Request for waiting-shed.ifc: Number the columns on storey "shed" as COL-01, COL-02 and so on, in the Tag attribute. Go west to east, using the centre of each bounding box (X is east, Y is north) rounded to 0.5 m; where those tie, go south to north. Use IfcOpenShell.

First a look at what the model holds.

```python
import ifcopenshell
import ifcopenshell.util.element
import ifcopenshell.util.placement

model = ifcopenshell.open("waiting-shed.ifc")
print(model.schema)
storey = next(s for s in model.by_type("IfcBuildingStorey") if s.Name == "shed")
columns = [e for e in ifcopenshell.util.element.get_decomposition(storey) if e.is_a("IfcColumn")]
for e in sorted(columns, key=lambda e: e.id()):
    origin = ifcopenshell.util.placement.get_local_placement(e.ObjectPlacement)[:3, 3]
    print(e.id(), e.Tag, e.Name, origin.round(2) + 0.0, sep=" | ")
```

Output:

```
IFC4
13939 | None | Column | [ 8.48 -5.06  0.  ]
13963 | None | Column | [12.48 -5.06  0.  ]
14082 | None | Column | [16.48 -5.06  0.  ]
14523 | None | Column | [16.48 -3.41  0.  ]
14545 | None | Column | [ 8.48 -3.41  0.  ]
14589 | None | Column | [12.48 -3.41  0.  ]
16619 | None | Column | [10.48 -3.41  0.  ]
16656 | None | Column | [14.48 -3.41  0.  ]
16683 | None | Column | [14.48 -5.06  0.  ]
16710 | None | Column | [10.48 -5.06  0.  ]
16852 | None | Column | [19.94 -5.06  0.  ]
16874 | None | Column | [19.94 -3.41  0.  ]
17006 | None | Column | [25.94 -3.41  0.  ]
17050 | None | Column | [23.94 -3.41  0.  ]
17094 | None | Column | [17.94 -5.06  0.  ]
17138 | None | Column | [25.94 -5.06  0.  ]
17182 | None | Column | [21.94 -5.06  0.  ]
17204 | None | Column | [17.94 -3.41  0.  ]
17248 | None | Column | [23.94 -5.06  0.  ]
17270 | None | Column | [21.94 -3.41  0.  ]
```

```python
import ifcopenshell
import ifcopenshell.geom
import ifcopenshell.util.element
import ifcopenshell.util.shape

model = ifcopenshell.open("waiting-shed.ifc")
settings = ifcopenshell.geom.settings()
settings.set("use-world-coords", True)


def centre(element):
    shape = ifcopenshell.geom.create_shape(settings, element)
    return ifcopenshell.util.shape.get_bbox_centroid(shape.geometry)


storey = next(s for s in model.by_type("IfcBuildingStorey") if s.Name == "shed")
columns = [e for e in ifcopenshell.util.element.get_decomposition(storey) if e.is_a("IfcColumn")]

# Insertion points can sit at a corner or the storey origin, so sort by the geometry (in metres).
centres = {e: centre(e) for e in columns}
columns.sort(key=lambda e: (round(centres[e][0] / 0.5), centres[e][1]))

for i, e in enumerate(columns, start=1):
    number = f"COL-{i:02d}"
    e.Tag = number
    print(e.id(), number)

model.write("waiting-shed_updated.ifc")
```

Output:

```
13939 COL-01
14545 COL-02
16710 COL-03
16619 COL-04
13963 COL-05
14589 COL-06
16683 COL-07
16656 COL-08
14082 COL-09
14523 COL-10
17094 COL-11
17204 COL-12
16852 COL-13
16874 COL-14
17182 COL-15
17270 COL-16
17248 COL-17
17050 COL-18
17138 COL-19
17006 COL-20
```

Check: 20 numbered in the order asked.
